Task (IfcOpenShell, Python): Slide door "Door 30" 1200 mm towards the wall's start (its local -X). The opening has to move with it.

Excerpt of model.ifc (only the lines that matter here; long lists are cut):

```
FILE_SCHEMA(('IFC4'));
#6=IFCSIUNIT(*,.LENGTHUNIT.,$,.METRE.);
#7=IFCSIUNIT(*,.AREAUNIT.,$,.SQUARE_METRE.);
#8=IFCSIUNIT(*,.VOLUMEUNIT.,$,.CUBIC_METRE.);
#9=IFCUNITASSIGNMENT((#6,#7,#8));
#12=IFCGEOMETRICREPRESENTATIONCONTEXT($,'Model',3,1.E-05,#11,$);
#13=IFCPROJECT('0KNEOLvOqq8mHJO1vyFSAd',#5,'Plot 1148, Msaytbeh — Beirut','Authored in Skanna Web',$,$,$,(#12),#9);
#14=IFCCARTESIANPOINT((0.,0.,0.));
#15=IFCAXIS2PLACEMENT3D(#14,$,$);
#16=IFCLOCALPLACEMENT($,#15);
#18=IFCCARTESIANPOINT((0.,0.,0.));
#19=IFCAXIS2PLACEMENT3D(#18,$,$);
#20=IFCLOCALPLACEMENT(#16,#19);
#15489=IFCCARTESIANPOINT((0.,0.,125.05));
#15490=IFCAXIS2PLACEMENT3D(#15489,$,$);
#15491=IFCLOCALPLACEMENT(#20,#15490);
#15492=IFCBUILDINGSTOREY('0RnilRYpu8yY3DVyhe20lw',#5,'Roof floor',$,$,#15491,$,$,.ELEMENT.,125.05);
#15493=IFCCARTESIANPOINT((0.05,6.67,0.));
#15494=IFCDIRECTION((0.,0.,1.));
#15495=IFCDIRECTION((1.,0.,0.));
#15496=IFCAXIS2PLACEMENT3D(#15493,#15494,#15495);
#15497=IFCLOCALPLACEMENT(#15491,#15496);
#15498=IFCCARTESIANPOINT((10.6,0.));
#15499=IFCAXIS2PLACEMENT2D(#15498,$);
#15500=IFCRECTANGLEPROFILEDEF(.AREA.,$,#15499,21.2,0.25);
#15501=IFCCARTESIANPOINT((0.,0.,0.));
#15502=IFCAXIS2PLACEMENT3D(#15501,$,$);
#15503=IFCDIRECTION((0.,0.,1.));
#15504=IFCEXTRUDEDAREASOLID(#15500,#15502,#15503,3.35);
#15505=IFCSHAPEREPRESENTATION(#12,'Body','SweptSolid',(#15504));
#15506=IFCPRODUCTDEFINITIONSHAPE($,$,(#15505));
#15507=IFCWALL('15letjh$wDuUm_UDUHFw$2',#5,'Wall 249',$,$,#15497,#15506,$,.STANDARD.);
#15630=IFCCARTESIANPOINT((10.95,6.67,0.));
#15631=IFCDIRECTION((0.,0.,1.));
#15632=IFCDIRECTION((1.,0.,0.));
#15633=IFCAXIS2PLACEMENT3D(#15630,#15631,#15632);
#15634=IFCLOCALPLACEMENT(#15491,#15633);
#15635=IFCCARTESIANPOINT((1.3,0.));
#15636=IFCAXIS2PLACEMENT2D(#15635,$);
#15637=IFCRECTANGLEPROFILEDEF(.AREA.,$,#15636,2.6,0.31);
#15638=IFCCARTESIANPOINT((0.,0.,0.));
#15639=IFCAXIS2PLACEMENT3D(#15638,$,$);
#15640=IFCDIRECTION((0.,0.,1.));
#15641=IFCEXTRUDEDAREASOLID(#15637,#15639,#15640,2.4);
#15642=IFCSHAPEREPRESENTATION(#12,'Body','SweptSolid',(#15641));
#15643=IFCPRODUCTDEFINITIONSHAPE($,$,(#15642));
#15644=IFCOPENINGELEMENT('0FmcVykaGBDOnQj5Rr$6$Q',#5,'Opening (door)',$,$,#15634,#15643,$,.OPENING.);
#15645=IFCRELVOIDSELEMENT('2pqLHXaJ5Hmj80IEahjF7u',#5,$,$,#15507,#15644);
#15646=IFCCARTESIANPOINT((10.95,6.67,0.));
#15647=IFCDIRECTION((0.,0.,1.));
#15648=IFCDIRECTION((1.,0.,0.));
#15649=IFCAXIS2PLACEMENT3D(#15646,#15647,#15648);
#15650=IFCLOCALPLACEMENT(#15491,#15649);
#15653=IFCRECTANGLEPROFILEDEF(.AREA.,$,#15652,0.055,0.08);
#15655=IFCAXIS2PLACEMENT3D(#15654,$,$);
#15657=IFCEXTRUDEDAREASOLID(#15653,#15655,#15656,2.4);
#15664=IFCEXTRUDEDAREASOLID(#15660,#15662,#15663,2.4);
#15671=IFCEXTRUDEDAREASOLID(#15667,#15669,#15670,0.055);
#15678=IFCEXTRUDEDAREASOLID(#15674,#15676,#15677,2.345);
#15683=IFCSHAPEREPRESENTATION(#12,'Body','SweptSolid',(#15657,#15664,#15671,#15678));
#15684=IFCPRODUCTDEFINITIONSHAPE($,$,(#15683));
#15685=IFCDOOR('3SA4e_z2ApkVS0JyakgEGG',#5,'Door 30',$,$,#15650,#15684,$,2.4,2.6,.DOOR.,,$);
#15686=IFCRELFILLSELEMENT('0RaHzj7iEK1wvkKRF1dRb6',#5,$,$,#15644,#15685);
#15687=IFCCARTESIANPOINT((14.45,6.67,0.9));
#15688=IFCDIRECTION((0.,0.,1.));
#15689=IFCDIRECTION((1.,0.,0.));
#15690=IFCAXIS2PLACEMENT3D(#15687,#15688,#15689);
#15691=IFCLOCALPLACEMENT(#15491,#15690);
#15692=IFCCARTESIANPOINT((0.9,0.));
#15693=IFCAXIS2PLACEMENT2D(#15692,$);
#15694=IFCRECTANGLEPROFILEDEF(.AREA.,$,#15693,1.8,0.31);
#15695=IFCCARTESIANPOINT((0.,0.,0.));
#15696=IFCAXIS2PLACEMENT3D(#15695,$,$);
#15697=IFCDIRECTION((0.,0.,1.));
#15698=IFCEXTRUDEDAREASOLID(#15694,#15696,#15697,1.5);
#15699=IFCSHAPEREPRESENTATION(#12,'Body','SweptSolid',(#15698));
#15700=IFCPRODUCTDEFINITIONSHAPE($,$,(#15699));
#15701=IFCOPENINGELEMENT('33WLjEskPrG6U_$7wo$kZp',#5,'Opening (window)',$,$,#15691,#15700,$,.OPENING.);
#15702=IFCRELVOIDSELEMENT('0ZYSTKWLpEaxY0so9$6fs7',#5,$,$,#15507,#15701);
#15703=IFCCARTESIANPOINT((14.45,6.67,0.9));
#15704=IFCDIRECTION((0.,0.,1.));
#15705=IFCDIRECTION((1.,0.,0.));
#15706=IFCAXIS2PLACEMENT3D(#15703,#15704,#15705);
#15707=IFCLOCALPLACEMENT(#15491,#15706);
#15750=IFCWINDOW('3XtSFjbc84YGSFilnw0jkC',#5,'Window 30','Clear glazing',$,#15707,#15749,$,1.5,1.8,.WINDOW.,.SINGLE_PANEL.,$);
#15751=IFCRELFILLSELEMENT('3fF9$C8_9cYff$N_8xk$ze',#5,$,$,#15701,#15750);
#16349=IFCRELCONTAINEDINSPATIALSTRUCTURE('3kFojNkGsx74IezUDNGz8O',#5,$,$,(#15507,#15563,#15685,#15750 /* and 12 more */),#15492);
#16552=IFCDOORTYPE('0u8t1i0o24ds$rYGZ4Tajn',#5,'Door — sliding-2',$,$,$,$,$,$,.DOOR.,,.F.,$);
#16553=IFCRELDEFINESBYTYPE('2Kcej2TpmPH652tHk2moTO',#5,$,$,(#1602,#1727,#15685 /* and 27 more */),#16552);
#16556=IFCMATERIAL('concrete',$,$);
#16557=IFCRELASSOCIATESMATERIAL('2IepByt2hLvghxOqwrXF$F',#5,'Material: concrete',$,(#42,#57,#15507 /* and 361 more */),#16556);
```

```python
import ifcopenshell
import ifcopenshell.api.geometry
import ifcopenshell.util.placement

model = ifcopenshell.open("model.ifc")

door = model.by_guid("3SA4e_z2ApkVS0JyakgEGG")
opening = door.FillsVoids[0].RelatingOpeningElement
wall = opening.VoidsElements[0].RelatingBuildingElement

wall_matrix = ifcopenshell.util.placement.get_local_placement(wall.ObjectPlacement)
shift = wall_matrix[:3, 0] * -1.2
before = ifcopenshell.util.placement.get_local_placement(door.ObjectPlacement)[:3, 3].copy()

# The door is not placed relative to its opening, so move both.
for product in (opening, door):
    matrix = ifcopenshell.util.placement.get_local_placement(product.ObjectPlacement)
    matrix[:3, 3] += shift
    ifcopenshell.api.geometry.edit_object_placement(model, product=product, matrix=matrix, is_si=False)

after = ifcopenshell.util.placement.get_local_placement(door.ObjectPlacement)[:3, 3]
print("door moved by", (after - before).round(3) + 0.0)

model.write("model_v2.ifc")
```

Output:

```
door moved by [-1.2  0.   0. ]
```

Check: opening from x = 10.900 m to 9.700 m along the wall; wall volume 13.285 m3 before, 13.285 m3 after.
